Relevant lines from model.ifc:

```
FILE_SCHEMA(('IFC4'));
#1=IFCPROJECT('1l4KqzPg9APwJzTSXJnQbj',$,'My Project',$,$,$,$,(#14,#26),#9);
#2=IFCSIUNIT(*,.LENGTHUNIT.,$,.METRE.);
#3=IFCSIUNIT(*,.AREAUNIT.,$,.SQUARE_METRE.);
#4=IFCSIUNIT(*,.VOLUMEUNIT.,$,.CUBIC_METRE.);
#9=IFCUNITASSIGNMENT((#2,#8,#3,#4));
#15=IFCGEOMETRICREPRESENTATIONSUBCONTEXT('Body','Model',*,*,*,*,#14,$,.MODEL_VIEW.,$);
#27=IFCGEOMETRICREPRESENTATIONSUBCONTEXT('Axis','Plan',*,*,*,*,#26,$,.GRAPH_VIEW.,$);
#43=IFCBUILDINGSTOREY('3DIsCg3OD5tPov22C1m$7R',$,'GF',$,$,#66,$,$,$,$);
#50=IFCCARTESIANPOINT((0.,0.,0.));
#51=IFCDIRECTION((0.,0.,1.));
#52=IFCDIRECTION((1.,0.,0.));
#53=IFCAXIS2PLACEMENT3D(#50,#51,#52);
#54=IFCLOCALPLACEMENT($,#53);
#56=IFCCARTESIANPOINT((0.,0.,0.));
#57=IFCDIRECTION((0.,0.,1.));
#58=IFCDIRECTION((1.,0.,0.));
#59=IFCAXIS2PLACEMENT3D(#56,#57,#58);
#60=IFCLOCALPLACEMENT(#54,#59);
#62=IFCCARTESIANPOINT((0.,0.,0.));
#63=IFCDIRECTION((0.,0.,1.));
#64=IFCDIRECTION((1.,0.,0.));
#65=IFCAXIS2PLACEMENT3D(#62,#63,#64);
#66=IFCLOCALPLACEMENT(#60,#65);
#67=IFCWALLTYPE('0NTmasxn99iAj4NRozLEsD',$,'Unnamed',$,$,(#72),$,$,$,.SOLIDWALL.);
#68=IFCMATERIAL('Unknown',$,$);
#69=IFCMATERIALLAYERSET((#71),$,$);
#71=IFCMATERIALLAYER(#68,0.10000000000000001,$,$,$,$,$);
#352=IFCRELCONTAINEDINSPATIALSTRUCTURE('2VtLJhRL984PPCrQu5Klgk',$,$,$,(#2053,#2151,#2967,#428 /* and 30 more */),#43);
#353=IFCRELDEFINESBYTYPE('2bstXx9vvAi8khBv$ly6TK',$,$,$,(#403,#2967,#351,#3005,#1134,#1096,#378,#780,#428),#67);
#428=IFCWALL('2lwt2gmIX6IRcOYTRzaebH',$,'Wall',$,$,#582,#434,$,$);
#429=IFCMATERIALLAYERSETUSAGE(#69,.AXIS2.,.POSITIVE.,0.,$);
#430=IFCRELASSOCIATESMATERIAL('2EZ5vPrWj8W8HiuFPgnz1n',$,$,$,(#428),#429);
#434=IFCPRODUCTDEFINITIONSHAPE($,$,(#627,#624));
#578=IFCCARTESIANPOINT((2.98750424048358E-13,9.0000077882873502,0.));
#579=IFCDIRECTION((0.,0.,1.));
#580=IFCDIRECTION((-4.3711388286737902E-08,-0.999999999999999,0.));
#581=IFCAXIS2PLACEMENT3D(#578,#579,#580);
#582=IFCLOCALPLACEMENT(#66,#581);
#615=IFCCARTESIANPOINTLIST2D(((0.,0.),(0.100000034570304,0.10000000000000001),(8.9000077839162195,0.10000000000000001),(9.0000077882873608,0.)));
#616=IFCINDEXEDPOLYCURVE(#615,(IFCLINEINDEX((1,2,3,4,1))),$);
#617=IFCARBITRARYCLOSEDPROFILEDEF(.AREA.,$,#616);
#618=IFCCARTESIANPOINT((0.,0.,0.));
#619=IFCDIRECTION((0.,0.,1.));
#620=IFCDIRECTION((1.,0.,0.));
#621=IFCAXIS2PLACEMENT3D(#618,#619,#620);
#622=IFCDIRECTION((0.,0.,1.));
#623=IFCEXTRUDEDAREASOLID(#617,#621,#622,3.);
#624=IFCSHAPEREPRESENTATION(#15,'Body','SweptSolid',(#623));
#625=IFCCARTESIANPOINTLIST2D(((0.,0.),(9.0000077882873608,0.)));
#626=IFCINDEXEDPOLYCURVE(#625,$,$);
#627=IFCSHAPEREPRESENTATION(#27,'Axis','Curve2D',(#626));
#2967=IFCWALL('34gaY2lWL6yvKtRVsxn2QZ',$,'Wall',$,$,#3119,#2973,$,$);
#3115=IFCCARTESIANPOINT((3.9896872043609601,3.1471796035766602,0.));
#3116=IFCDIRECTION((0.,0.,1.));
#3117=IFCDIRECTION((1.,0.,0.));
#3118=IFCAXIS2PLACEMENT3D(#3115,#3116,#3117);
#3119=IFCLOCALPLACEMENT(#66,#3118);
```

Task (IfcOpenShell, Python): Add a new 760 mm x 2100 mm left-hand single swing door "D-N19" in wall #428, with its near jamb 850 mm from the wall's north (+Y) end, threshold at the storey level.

```python
import numpy as np
import ifcopenshell
import ifcopenshell.api.feature
import ifcopenshell.api.geometry
import ifcopenshell.api.root
import ifcopenshell.api.spatial
import ifcopenshell.geom
import ifcopenshell.util.element
import ifcopenshell.util.placement
import ifcopenshell.util.representation
import ifcopenshell.util.shape
import ifcopenshell.util.unit

model = ifcopenshell.open("model.ifc")
unit_scale = ifcopenshell.util.unit.calculate_unit_scale(model)
settings = ifcopenshell.geom.settings()


def volume(element):
    """Net volume in cubic metres, openings subtracted."""
    shape = ifcopenshell.geom.create_shape(settings, element)
    return ifcopenshell.util.shape.get_volume(shape.geometry)


wall = model.by_guid("2lwt2gmIX6IRcOYTRzaebH")
storey = ifcopenshell.util.element.get_container(wall, ifc_class="IfcBuildingStorey")
context = ifcopenshell.util.representation.get_context(model, "Model", "Body", "MODEL_VIEW")
before = volume(wall)

width, height, from_end, sill = 0.76, 2.1, 0.85, 0.0  # metres

# The wall runs along its own X axis, and the end named is its -X end.
wall_shape = ifcopenshell.geom.create_shape(settings, wall)
x, y, z = ifcopenshell.util.shape.get_vertices(wall_shape.geometry).T
start = x.min() + from_end
face, thickness = float(y.min()), float(y.max() - y.min())
wall_matrix = ifcopenshell.util.placement.get_local_placement(wall.ObjectPlacement)
level = ifcopenshell.util.placement.get_local_placement(storey.ObjectPlacement)[2, 3]


def in_wall(x, y):
    """Placement at x, y metres in the wall's axes, at sill height."""
    matrix = wall_matrix.copy()
    matrix[:, 3] = wall_matrix @ np.array([x / unit_scale, y / unit_scale, 0.0, 1.0])
    matrix[2, 3] = level + sill / unit_scale
    return matrix


# Opening: a box that overshoots both wall faces by 50 mm.
opening = ifcopenshell.api.root.create_entity(model, ifc_class="IfcOpeningElement", predefined_type="OPENING")
box = ifcopenshell.api.geometry.add_wall_representation(
    model, context=context, length=width, height=height, thickness=thickness + 0.1
)
ifcopenshell.api.geometry.assign_representation(model, product=opening, representation=box)
ifcopenshell.api.geometry.edit_object_placement(model, product=opening, matrix=in_wall(start, face - 0.05), is_si=False)
ifcopenshell.api.feature.add_feature(model, feature=opening, element=wall)

door = ifcopenshell.api.root.create_entity(model, ifc_class="IfcDoor", name="D-N19", predefined_type="DOOR")
door.OverallWidth, door.OverallHeight = width / unit_scale, height / unit_scale
door.OperationType = "SINGLE_SWING_LEFT"
body = ifcopenshell.api.geometry.add_door_representation(
    model,
    context=context,
    overall_width=door.OverallWidth,
    overall_height=door.OverallHeight,
    operation_type="SINGLE_SWING_LEFT",
    lining_properties={"LiningDepth": thickness / unit_scale, "ThresholdDepth": thickness / unit_scale},
)
ifcopenshell.api.geometry.assign_representation(model, product=door, representation=body)
ifcopenshell.api.spatial.assign_container(model, products=[door], relating_structure=storey)
ifcopenshell.api.feature.add_filling(model, opening=opening, element=door)

# The lining spans the wall, so the door starts at the wall face.
ifcopenshell.api.geometry.edit_object_placement(model, product=door, matrix=in_wall(start, face), is_si=False)

after = volume(wall)

print(f"wall volume {before:.3f} -> {after:.3f} m3")

model.write("model-out.ifc")
```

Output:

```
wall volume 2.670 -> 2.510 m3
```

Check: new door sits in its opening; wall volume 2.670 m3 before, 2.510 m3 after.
